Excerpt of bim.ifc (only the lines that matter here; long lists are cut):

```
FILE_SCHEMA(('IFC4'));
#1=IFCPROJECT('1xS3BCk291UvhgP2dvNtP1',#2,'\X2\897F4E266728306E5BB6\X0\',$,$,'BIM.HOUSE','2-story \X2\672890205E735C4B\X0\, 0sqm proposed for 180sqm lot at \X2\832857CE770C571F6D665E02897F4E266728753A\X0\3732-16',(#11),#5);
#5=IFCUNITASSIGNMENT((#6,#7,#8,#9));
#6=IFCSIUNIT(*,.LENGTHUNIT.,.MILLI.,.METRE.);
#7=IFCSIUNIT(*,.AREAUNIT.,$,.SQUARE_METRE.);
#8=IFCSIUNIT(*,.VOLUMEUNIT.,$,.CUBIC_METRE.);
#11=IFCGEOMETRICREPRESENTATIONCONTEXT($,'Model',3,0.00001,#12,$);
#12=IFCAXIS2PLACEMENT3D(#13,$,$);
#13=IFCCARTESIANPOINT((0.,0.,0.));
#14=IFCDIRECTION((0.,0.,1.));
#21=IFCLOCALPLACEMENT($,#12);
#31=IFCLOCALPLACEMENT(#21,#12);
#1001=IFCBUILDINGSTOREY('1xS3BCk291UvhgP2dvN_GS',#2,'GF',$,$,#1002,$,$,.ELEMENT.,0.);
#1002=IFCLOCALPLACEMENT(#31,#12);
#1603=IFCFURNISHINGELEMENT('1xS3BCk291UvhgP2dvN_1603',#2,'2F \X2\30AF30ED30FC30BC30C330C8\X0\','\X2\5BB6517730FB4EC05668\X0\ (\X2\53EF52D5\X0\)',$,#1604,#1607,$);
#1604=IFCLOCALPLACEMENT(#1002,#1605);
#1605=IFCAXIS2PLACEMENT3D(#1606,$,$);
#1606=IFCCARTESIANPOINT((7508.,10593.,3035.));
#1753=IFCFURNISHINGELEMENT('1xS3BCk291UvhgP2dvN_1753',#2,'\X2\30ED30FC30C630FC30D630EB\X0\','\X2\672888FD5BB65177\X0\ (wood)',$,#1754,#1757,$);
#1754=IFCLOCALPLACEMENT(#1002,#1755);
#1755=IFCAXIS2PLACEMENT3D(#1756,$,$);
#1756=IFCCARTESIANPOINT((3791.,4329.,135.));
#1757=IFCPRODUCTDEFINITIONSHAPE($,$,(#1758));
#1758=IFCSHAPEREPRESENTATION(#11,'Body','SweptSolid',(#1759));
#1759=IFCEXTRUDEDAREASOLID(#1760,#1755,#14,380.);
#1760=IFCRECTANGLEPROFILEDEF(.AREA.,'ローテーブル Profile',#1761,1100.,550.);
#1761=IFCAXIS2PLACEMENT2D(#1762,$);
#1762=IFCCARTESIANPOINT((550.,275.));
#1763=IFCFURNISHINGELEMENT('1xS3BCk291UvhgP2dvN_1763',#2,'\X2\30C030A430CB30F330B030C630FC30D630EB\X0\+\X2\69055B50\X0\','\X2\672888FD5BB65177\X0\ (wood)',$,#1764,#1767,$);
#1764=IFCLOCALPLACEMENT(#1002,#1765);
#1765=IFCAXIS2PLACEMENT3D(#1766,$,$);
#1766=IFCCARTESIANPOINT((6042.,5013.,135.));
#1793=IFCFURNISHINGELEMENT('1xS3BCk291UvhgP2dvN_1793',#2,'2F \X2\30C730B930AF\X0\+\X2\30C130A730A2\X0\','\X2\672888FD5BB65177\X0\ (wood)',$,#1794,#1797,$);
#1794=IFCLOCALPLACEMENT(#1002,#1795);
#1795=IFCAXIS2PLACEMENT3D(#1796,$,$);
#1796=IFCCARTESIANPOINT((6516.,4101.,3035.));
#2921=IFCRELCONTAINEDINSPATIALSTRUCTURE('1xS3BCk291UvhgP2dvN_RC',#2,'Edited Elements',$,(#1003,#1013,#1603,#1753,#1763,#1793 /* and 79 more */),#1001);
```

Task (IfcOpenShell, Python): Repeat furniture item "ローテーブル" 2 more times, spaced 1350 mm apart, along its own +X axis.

```python
import ifcopenshell
import ifcopenshell.api.geometry
import ifcopenshell.api.root
import ifcopenshell.util.element
import ifcopenshell.util.placement
import ifcopenshell.util.unit

model = ifcopenshell.open("bim.ifc")
unit_scale = ifcopenshell.util.unit.calculate_unit_scale(model)


def reuse_history(source, copy):
    """copy_class also copies each property set's owner history, people and application; keep the originals."""
    for rel in copy.IsDefinedBy:
        if rel.is_a("IfcRelDefinesByProperties") and (history := rel.RelatingPropertyDefinition.OwnerHistory):
            rel.RelatingPropertyDefinition.OwnerHistory = source.OwnerHistory
            ifcopenshell.util.element.remove_deep2(model, history)


source = model.by_id(1753)
base = ifcopenshell.util.placement.get_local_placement(source.ObjectPlacement)
step = base[:3, 0] * 1.35 / unit_scale

for i in range(1, 3):
    copy = ifcopenshell.api.root.copy_class(model, product=source)
    copy.Representation = ifcopenshell.util.element.copy_deep(
        model, source.Representation, exclude=["IfcGeometricRepresentationContext", "IfcRepresentationMap"]
    )
    reuse_history(source, copy)
    matrix = base.copy()
    matrix[:3, 3] += i * step
    print("added at", matrix[:3, 3].round(3) + 0.0)
    ifcopenshell.api.geometry.edit_object_placement(model, product=copy, matrix=matrix, is_si=False)

model.write("bim_rev.ifc")
```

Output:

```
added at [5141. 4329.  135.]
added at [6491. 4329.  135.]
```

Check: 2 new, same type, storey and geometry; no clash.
